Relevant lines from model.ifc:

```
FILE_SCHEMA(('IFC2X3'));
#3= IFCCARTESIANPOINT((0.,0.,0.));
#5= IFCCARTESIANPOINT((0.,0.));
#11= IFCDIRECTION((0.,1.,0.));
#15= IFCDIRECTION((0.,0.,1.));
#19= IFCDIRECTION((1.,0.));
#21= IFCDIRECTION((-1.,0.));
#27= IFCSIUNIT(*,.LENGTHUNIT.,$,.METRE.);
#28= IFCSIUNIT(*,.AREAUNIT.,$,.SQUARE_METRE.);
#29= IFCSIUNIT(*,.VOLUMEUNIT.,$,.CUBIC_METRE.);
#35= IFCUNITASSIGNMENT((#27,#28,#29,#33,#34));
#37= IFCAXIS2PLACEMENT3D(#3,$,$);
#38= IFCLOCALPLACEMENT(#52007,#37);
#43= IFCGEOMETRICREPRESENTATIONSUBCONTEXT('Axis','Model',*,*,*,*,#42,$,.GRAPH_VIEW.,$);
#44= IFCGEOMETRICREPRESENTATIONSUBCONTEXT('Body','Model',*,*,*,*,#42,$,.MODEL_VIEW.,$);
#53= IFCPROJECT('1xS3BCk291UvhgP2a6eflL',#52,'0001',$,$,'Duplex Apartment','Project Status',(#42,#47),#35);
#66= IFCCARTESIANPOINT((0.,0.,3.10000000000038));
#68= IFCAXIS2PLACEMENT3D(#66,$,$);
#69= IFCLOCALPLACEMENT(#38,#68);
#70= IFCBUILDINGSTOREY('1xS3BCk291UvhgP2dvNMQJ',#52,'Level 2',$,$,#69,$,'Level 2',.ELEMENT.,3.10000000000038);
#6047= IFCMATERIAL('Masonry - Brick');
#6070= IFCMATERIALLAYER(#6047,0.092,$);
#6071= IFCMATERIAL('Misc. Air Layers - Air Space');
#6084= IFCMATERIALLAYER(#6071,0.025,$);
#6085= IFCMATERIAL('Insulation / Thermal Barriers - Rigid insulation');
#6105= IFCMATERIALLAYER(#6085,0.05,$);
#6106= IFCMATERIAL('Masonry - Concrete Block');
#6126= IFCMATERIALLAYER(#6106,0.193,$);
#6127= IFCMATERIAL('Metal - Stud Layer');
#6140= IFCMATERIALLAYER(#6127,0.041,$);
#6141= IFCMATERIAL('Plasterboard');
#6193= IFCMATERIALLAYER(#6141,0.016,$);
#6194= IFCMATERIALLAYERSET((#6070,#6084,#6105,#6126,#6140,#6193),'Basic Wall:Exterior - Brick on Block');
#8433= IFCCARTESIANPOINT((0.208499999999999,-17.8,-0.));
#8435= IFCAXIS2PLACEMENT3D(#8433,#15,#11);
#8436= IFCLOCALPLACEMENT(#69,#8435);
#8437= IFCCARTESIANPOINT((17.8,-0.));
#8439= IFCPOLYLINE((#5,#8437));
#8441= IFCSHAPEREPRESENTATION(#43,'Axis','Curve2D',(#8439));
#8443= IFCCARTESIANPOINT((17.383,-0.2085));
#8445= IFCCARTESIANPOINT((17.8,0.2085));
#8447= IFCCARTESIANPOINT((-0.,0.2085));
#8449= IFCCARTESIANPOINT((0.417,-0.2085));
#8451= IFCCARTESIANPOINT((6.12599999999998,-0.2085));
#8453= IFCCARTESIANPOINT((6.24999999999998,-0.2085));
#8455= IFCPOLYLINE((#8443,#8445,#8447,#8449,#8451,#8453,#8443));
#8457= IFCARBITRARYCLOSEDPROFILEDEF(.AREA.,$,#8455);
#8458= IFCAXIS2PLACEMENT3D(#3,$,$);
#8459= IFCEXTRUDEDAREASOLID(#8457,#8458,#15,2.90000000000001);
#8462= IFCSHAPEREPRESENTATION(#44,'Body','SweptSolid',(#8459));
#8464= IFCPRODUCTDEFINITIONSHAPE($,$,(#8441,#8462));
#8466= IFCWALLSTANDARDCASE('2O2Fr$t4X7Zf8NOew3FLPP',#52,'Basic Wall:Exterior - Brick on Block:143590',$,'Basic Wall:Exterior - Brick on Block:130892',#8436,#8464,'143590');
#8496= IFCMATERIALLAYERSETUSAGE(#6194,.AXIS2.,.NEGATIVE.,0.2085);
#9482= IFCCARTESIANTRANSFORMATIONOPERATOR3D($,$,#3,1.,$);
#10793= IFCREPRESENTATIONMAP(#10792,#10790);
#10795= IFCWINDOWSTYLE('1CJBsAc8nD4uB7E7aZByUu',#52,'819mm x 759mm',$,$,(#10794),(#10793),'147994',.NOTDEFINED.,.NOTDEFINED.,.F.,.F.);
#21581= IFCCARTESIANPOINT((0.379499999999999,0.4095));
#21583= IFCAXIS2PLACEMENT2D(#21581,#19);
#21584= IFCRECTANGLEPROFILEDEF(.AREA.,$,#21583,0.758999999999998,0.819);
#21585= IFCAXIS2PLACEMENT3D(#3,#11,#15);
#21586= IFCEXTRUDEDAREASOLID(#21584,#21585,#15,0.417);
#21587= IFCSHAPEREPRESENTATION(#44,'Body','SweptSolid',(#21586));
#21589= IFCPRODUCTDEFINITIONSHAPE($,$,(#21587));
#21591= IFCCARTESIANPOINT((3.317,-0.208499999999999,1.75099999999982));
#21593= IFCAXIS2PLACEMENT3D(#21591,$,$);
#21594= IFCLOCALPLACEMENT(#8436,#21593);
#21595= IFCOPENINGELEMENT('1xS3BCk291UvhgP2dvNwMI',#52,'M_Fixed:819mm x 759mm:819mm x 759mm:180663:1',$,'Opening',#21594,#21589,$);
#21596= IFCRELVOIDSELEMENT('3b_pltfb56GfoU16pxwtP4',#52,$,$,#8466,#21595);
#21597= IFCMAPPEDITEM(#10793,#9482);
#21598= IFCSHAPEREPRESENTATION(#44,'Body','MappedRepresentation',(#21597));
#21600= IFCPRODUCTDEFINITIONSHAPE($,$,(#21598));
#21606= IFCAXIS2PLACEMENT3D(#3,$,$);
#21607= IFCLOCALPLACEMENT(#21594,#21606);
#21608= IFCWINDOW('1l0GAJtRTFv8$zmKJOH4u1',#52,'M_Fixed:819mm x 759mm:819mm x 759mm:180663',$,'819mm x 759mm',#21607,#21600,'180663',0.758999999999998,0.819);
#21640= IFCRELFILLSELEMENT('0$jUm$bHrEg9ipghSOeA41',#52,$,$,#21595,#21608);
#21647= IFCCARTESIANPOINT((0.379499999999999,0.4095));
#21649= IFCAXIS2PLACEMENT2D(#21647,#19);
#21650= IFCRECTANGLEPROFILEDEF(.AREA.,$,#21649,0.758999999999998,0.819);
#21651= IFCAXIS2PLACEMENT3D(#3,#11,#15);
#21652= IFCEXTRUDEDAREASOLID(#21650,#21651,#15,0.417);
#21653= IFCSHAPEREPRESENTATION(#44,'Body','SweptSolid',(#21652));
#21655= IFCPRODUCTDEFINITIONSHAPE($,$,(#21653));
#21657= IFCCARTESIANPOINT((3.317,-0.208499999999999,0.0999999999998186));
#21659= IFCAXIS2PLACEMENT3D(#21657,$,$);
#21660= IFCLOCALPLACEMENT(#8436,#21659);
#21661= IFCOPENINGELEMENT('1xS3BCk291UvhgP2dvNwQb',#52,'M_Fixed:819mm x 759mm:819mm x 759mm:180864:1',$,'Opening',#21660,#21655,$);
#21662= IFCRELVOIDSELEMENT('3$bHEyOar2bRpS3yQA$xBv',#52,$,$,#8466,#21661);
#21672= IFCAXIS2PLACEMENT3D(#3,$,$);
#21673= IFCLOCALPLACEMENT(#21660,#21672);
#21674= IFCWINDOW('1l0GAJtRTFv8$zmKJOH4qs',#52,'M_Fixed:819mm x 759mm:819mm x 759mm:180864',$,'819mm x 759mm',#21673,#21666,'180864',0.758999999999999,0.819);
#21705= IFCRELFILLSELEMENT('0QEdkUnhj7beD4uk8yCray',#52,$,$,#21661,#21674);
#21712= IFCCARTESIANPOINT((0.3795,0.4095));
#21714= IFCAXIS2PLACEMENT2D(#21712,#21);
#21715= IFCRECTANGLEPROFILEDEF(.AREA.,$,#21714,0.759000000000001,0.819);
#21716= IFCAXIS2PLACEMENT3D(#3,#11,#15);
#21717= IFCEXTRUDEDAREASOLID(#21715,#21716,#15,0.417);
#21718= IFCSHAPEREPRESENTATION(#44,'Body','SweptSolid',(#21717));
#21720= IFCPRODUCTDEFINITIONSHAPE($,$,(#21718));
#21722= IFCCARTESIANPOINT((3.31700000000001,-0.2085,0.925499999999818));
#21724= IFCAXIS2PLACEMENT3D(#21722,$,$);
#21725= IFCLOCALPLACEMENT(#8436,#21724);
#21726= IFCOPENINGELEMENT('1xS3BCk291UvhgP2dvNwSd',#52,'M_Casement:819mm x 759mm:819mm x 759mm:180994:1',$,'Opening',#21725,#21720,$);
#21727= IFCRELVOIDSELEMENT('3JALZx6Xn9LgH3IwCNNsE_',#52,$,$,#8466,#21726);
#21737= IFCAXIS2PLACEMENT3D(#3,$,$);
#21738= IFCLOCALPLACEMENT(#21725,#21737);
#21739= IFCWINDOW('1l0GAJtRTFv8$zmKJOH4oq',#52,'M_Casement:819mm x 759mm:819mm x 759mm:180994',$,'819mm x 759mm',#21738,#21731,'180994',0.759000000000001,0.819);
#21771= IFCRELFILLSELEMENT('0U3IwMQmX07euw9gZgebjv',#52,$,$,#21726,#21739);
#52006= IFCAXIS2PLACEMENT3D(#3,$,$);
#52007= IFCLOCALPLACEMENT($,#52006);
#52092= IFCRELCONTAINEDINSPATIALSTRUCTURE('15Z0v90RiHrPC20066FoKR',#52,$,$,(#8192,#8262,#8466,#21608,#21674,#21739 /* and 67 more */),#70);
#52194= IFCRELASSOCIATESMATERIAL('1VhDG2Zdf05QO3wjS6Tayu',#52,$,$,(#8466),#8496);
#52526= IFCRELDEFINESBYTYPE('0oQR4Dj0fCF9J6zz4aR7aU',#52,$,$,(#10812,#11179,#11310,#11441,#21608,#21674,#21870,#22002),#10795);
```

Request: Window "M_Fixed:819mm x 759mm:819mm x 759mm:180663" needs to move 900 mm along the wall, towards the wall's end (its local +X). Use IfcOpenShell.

```python
import ifcopenshell
import ifcopenshell.api.geometry
import ifcopenshell.util.placement

model = ifcopenshell.open("model.ifc")

window = model.by_id(21608)
opening = window.FillsVoids[0].RelatingOpeningElement
wall = opening.VoidsElements[0].RelatingBuildingElement

wall_matrix = ifcopenshell.util.placement.get_local_placement(wall.ObjectPlacement)
shift = wall_matrix[:3, 0] * 0.9
before = ifcopenshell.util.placement.get_local_placement(window.ObjectPlacement)[:3, 3].copy()

# The window is placed relative to its opening, so it follows when the opening moves.
matrix = ifcopenshell.util.placement.get_local_placement(opening.ObjectPlacement)
matrix[:3, 3] += shift
ifcopenshell.api.geometry.edit_object_placement(
    model, product=opening, matrix=matrix, is_si=False, should_transform_children=True
)

after = ifcopenshell.util.placement.get_local_placement(window.ObjectPlacement)[:3, 3]
print("window moved by", (after - before).round(3) + 0.0)

model.write("model-out.ifc")
```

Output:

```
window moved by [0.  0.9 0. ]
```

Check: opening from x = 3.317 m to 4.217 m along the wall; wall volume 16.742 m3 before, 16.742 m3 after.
